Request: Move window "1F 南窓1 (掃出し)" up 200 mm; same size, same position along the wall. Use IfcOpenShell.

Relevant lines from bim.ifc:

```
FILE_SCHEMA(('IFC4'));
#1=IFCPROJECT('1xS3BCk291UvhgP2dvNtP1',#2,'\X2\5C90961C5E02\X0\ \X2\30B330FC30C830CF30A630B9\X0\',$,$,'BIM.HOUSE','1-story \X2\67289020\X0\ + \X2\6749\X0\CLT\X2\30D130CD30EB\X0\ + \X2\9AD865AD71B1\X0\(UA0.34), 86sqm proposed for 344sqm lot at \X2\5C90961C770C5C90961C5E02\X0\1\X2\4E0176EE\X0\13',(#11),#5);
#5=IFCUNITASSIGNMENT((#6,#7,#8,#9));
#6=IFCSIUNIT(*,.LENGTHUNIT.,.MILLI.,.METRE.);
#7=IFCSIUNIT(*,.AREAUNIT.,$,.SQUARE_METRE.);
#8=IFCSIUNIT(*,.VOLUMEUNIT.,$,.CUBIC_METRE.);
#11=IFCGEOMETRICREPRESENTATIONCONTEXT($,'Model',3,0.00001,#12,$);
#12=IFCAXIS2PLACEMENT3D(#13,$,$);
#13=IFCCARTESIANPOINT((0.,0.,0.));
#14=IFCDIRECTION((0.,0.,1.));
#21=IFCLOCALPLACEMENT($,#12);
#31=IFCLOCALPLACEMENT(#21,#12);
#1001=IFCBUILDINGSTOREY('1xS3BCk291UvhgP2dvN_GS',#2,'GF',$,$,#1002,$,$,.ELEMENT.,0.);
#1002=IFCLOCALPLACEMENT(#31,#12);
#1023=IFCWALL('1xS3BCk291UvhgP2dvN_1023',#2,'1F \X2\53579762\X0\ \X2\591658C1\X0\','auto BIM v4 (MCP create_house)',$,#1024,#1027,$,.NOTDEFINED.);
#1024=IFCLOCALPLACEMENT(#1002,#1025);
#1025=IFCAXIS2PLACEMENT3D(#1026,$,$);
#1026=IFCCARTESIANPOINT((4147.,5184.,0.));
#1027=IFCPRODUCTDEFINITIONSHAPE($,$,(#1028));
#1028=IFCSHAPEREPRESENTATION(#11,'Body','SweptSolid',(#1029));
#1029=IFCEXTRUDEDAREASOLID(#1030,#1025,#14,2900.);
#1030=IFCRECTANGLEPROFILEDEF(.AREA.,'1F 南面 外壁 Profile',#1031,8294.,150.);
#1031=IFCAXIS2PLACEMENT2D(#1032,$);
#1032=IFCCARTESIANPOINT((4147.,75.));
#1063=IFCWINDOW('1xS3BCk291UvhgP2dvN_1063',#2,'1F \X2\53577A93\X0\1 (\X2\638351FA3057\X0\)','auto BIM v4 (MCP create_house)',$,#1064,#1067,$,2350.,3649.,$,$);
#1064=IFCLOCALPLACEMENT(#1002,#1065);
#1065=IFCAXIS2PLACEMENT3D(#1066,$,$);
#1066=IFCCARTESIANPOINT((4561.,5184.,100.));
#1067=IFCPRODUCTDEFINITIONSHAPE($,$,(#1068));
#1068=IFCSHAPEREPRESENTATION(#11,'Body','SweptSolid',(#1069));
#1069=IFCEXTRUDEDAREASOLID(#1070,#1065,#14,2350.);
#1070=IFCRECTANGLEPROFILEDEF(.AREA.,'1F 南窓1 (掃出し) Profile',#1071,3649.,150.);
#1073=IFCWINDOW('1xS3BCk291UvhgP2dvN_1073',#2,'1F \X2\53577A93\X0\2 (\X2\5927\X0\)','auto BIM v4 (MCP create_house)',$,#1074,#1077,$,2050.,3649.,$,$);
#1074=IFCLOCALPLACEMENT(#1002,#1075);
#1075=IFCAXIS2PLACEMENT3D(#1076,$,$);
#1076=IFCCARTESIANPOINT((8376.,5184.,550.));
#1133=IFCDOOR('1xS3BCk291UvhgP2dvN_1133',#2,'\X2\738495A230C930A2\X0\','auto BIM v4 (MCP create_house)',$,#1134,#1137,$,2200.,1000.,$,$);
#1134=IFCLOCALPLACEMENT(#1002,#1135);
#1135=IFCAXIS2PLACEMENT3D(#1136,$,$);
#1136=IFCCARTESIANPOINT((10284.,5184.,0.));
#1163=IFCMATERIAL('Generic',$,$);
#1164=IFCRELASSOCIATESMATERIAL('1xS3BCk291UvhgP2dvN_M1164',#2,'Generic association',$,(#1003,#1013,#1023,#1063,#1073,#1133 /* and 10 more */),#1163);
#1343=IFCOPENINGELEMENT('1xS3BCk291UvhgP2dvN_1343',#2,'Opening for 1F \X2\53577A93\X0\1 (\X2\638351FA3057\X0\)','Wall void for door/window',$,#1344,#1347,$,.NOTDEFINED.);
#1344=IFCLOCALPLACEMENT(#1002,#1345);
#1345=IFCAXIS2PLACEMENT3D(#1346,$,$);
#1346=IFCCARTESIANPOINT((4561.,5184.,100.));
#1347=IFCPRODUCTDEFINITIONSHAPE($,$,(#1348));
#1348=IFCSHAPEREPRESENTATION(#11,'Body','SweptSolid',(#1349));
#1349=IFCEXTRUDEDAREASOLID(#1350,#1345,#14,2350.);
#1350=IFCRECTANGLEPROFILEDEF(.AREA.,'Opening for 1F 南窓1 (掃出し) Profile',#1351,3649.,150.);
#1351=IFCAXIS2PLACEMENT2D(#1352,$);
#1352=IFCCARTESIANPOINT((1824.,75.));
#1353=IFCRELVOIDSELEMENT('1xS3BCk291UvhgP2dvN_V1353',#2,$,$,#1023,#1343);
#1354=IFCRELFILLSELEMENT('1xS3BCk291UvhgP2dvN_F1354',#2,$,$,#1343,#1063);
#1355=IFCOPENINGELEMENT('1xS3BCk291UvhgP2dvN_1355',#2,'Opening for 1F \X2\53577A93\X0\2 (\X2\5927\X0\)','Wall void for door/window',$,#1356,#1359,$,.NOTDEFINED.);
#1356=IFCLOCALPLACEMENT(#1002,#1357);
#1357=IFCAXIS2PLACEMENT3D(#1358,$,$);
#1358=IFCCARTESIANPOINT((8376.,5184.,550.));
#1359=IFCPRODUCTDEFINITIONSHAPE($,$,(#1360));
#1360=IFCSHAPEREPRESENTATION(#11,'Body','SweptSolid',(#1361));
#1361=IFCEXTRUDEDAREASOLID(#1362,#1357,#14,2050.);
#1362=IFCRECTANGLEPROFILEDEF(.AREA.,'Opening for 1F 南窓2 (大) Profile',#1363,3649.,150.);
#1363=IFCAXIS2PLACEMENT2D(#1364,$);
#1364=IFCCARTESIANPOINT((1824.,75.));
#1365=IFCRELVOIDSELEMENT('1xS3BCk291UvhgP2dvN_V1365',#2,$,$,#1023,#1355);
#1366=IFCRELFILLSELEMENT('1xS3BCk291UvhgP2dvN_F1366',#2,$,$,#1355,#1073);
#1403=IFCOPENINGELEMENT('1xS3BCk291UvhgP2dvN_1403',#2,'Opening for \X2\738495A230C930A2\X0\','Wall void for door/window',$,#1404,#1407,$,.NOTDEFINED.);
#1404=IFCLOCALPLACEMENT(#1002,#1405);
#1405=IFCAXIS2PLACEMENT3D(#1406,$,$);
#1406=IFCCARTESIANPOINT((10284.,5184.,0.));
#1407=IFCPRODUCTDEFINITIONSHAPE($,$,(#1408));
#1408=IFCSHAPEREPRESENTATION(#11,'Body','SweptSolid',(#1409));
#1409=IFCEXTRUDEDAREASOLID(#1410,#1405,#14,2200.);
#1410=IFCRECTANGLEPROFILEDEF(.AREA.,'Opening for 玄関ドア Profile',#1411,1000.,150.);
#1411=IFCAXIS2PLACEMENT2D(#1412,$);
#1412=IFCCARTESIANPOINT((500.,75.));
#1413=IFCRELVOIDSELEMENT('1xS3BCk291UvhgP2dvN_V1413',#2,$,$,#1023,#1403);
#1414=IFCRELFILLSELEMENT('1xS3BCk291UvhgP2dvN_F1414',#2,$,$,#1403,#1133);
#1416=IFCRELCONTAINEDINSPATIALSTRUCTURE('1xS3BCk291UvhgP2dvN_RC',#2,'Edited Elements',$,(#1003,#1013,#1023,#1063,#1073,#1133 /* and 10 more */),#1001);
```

```python
import numpy as np
import ifcopenshell
import ifcopenshell.api.geometry
import ifcopenshell.util.placement
import ifcopenshell.util.unit

model = ifcopenshell.open("bim.ifc")
unit_scale = ifcopenshell.util.unit.calculate_unit_scale(model)

window = model.by_guid("1xS3BCk291UvhgP2dvN_1063")
opening = window.FillsVoids[0].RelatingOpeningElement
dz = 0.2 / unit_scale

shift = np.array([0.0, 0.0, dz])
# The window is not placed relative to its opening, so move both.
for product in (opening, window):
    matrix = ifcopenshell.util.placement.get_local_placement(product.ObjectPlacement)
    matrix[:3, 3] += shift
    ifcopenshell.api.geometry.edit_object_placement(model, product=product, matrix=matrix, is_si=False)

print(f"moved by {dz * unit_scale:+.3f} m")

model.write("bim-out.ifc")
```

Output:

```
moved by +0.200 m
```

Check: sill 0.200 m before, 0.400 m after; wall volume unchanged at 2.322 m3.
